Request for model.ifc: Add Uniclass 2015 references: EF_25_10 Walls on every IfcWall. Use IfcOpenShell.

First a look at what the model holds.

```python
import ifcopenshell

model = ifcopenshell.open("model.ifc")
print(model.schema)
print("classifications:", [c.Name for c in model.by_type("IfcClassification")])
for ifc_class in ("IfcDoor", "IfcRoof", "IfcStair", "IfcWall", "IfcWindow"):
    print(ifc_class, len(model.by_type(ifc_class)))
```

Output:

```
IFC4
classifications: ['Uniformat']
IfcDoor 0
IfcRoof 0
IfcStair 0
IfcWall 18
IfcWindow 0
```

```python
import ifcopenshell
import ifcopenshell.api.classification

model = ifcopenshell.open("model.ifc")

system = ifcopenshell.api.classification.add_classification(model, classification="Uniclass 2015")

codes = {
    "IfcWall": ("EF_25_10", "Walls"),
}
for ifc_class, (code, name) in codes.items():
    products = model.by_type(ifc_class)
    ifcopenshell.api.classification.add_reference(
        model, products=products, classification=system, identification=code, name=name
    )
    print(code, len(products))

model.write("model_updated.ifc")
```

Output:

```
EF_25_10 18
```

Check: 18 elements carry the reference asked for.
